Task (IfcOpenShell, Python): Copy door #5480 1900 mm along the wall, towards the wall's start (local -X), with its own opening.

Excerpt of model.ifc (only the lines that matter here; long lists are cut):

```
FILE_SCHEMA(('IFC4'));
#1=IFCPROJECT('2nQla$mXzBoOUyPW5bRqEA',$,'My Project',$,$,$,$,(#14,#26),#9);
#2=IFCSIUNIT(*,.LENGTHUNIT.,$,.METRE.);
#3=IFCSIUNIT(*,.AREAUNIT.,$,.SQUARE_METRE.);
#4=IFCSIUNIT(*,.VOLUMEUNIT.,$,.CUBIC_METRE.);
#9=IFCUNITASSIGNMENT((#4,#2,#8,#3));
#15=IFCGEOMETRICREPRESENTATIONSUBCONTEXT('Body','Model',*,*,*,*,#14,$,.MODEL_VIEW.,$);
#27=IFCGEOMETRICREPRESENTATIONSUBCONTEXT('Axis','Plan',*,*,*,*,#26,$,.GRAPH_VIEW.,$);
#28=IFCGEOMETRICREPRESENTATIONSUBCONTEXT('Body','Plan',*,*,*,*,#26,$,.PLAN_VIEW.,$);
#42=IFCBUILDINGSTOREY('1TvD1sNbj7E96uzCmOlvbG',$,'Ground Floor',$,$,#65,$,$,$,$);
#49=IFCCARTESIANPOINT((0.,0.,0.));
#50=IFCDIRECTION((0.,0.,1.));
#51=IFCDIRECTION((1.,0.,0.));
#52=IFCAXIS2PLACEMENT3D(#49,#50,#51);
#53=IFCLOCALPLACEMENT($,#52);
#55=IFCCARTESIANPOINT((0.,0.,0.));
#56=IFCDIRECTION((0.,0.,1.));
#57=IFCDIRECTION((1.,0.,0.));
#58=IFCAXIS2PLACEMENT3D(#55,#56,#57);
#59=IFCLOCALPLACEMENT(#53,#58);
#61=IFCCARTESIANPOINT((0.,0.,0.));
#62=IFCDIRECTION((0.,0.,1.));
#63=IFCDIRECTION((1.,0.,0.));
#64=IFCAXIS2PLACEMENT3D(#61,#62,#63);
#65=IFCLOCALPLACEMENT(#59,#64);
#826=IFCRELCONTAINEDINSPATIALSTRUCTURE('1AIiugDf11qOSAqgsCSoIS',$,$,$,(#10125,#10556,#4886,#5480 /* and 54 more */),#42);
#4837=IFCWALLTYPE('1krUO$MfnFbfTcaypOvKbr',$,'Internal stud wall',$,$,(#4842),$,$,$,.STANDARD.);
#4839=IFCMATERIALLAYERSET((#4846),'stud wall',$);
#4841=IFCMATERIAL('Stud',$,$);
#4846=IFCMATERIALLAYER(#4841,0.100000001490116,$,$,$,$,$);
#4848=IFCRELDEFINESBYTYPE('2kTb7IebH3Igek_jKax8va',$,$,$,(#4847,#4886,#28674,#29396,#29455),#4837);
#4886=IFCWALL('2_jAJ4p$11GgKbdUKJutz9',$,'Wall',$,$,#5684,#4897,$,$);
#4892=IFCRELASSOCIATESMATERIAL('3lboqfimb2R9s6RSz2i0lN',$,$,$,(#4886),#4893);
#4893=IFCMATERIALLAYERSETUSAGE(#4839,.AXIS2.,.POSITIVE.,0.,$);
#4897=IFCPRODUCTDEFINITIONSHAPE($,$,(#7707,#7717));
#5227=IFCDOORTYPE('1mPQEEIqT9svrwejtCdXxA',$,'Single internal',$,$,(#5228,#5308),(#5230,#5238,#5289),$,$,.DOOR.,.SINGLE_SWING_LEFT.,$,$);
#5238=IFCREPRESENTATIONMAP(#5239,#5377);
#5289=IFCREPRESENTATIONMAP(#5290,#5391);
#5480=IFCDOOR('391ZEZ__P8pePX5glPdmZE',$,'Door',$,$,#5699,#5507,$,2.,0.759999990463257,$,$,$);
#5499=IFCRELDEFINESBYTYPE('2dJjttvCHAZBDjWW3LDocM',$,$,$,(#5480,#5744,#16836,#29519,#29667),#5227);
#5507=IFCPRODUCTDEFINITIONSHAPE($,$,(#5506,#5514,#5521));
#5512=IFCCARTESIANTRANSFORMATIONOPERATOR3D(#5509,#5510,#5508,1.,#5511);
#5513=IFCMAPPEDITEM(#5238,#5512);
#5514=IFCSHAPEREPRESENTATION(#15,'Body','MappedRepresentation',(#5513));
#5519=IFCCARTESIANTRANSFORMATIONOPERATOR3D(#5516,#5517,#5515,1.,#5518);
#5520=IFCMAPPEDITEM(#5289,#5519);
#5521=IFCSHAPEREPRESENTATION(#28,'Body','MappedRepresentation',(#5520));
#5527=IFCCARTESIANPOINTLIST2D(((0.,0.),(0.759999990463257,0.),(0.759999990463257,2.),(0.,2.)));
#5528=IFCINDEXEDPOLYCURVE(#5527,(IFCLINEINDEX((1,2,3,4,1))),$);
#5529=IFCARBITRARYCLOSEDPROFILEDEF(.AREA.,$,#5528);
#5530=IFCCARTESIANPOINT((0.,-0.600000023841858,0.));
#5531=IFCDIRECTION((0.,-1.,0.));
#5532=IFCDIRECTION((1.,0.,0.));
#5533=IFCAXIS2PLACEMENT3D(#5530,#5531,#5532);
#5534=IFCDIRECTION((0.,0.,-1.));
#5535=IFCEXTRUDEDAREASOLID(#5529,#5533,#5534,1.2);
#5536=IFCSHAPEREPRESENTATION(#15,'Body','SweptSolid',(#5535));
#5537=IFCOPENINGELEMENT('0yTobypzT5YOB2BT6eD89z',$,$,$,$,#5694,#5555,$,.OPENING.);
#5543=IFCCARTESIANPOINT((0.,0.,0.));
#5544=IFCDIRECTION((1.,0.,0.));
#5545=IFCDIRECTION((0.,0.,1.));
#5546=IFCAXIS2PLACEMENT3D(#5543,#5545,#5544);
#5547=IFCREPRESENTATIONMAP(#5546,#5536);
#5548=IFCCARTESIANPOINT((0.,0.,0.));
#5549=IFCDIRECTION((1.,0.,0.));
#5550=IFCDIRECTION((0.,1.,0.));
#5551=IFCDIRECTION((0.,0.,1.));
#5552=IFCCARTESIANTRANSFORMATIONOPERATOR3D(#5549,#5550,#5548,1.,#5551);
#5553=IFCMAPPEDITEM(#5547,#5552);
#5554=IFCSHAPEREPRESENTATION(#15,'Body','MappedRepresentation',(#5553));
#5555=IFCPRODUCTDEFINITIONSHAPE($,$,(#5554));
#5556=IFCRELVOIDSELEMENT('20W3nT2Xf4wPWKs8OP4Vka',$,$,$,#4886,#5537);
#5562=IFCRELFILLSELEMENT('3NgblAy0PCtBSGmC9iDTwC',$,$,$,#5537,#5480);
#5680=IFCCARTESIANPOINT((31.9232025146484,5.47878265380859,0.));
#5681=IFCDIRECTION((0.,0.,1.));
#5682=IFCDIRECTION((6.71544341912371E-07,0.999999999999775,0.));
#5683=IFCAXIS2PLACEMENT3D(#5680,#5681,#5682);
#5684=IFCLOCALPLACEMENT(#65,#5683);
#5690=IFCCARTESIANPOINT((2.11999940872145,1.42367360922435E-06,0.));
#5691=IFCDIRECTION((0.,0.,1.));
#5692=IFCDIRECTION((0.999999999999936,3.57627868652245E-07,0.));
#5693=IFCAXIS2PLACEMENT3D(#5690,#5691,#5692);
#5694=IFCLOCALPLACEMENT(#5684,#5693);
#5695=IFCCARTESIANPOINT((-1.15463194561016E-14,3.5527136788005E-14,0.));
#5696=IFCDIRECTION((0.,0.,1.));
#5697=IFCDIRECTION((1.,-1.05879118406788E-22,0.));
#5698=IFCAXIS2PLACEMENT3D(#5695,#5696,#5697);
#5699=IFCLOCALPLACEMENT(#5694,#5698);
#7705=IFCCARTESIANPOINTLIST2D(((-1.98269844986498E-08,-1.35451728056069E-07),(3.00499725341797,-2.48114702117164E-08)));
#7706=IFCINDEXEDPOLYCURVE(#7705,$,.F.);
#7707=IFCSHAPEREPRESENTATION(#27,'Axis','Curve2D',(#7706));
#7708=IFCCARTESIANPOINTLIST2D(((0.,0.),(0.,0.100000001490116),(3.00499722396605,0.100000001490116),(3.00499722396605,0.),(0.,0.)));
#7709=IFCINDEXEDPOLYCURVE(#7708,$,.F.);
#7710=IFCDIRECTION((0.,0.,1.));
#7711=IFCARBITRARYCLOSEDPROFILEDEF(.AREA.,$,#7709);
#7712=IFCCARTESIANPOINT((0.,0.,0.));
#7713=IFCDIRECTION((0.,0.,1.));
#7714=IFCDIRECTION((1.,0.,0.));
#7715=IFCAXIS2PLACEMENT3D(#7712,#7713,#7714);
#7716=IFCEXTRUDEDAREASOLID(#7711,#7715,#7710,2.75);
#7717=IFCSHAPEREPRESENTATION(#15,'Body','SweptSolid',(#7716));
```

```python
import ifcopenshell
import ifcopenshell.api.feature
import ifcopenshell.api.geometry
import ifcopenshell.api.root
import ifcopenshell.geom
import ifcopenshell.util.element
import ifcopenshell.util.placement
import ifcopenshell.util.shape

model = ifcopenshell.open("model.ifc")
settings = ifcopenshell.geom.settings()


def volume(element):
    """Net volume in cubic metres, openings subtracted."""
    shape = ifcopenshell.geom.create_shape(settings, element)
    return ifcopenshell.util.shape.get_volume(shape.geometry)


door = model.by_id(5480)
opening = door.FillsVoids[0].RelatingOpeningElement
wall = opening.VoidsElements[0].RelatingBuildingElement
before = volume(wall)
shift = ifcopenshell.util.placement.get_local_placement(wall.ObjectPlacement)[:3, 0] * -1.9

# copy_class copies the void relationship, type, container and properties, but no geometry.
new_opening = ifcopenshell.api.root.copy_class(model, product=opening)
new_opening.Representation = ifcopenshell.util.element.copy_deep(
    model, opening.Representation, exclude=["IfcGeometricRepresentationContext", "IfcRepresentationMap"]
)
new_door = ifcopenshell.api.root.copy_class(model, product=door)
new_door.Representation = ifcopenshell.util.element.copy_deep(
    model, door.Representation, exclude=["IfcGeometricRepresentationContext", "IfcRepresentationMap"]
)
ifcopenshell.api.feature.add_filling(model, opening=new_opening, element=new_door)

for old, new in ((opening, new_opening), (door, new_door)):
    matrix = ifcopenshell.util.placement.get_local_placement(old.ObjectPlacement)
    matrix[:3, 3] += shift
    ifcopenshell.api.geometry.edit_object_placement(model, product=new, matrix=matrix, is_si=False)

after = volume(wall)

print(f"wall volume {before:.3f} -> {after:.3f} m3")

model.write("model_updated.ifc")
```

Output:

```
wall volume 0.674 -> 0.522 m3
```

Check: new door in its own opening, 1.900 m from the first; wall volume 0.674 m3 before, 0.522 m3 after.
